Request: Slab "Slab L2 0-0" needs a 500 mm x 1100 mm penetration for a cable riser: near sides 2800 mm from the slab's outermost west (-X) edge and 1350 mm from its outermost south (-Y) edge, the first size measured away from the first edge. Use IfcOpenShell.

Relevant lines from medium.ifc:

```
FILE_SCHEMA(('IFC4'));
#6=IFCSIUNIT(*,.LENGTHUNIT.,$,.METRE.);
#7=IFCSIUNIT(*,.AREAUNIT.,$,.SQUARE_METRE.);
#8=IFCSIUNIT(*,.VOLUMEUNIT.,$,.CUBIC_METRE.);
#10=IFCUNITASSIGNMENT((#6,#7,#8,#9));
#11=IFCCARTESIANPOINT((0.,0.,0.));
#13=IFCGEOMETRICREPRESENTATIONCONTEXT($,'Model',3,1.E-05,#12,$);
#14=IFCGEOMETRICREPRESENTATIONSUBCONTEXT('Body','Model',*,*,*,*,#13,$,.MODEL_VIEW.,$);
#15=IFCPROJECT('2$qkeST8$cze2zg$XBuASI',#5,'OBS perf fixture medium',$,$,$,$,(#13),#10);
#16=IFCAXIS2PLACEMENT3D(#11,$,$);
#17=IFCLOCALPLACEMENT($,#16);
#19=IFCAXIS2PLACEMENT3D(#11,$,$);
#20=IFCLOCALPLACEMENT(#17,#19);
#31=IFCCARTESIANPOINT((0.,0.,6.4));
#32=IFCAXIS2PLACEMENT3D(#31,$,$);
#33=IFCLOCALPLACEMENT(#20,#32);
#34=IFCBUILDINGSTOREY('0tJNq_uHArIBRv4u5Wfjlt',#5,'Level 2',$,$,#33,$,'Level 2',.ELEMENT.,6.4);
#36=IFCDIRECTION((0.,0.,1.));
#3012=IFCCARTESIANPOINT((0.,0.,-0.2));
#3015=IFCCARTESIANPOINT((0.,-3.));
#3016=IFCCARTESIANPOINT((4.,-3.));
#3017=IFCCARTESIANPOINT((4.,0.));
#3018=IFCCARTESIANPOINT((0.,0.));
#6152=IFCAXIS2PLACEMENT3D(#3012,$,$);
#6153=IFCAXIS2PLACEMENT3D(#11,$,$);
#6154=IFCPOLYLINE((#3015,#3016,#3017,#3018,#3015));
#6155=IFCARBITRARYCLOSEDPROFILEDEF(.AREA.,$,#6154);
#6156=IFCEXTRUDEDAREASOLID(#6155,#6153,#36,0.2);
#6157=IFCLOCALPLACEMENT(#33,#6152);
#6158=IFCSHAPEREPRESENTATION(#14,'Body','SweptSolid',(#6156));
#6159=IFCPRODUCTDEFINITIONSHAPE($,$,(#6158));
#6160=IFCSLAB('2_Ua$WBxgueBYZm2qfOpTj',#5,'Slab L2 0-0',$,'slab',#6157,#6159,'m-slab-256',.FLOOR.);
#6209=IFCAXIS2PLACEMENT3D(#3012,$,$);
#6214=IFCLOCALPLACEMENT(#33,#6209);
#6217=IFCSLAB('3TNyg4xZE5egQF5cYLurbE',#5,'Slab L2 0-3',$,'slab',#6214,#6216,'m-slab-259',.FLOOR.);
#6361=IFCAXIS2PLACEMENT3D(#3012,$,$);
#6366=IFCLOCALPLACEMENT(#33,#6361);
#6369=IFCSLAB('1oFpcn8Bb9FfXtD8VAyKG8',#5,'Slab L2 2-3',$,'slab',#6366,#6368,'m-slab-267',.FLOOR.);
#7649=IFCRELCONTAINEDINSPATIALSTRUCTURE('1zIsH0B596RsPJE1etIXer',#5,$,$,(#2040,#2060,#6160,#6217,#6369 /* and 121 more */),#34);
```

```python
import numpy as np
import ifcopenshell
import ifcopenshell.api.feature
import ifcopenshell.api.geometry
import ifcopenshell.api.root
import ifcopenshell.geom
import ifcopenshell.util.placement
import ifcopenshell.util.representation
import ifcopenshell.util.shape
import ifcopenshell.util.unit

model = ifcopenshell.open("medium.ifc")
unit_scale = ifcopenshell.util.unit.calculate_unit_scale(model)
settings = ifcopenshell.geom.settings()


def volume(element):
    """Net volume in cubic metres, openings subtracted."""
    shape = ifcopenshell.geom.create_shape(settings, element)
    return ifcopenshell.util.shape.get_volume(shape.geometry)


slab = model.by_guid("2_Ua$WBxgueBYZm2qfOpTj")
before = volume(slab)

# Extent in the slab's own axes, in metres. The edges named are its -X and -Y sides.
slab_shape = ifcopenshell.geom.create_shape(settings, slab)
vertices = ifcopenshell.util.shape.get_vertices(slab_shape.geometry)
x_min, y_min, bottom = vertices.min(axis=0)
top = vertices[:, 2].max()

opening = ifcopenshell.api.root.create_entity(model, ifc_class="IfcOpeningElement", name="Cable riser opening", predefined_type="OPENING")
context = ifcopenshell.util.representation.get_context(model, "Model", "Body", "MODEL_VIEW")
width, depth = 0.5, 1.1
outline = [(0.0, 0.0), (width, 0.0), (width, depth), (0.0, depth), (0.0, 0.0)]
# Overshoot both faces by 50 mm so the cut is clean.
shape = ifcopenshell.api.geometry.add_slab_representation(
    model, context=context, depth=top - bottom + 0.1, polyline=outline
)
ifcopenshell.api.geometry.assign_representation(model, product=opening, representation=shape)

matrix = ifcopenshell.util.placement.get_local_placement(slab.ObjectPlacement)
matrix[:, 3] = matrix @ np.append(np.array([x_min + 2.8, y_min + 1.35, bottom - 0.05]) / unit_scale, 1.0)
ifcopenshell.api.geometry.edit_object_placement(model, product=opening, matrix=matrix, is_si=False)
ifcopenshell.api.feature.add_feature(model, feature=opening, element=slab)

after = volume(slab)

print(f"slab volume {before:.3f} -> {after:.3f} m3")

model.write("medium_rev.ifc")
```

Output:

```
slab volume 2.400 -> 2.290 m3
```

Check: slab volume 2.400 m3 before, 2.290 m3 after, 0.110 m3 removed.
